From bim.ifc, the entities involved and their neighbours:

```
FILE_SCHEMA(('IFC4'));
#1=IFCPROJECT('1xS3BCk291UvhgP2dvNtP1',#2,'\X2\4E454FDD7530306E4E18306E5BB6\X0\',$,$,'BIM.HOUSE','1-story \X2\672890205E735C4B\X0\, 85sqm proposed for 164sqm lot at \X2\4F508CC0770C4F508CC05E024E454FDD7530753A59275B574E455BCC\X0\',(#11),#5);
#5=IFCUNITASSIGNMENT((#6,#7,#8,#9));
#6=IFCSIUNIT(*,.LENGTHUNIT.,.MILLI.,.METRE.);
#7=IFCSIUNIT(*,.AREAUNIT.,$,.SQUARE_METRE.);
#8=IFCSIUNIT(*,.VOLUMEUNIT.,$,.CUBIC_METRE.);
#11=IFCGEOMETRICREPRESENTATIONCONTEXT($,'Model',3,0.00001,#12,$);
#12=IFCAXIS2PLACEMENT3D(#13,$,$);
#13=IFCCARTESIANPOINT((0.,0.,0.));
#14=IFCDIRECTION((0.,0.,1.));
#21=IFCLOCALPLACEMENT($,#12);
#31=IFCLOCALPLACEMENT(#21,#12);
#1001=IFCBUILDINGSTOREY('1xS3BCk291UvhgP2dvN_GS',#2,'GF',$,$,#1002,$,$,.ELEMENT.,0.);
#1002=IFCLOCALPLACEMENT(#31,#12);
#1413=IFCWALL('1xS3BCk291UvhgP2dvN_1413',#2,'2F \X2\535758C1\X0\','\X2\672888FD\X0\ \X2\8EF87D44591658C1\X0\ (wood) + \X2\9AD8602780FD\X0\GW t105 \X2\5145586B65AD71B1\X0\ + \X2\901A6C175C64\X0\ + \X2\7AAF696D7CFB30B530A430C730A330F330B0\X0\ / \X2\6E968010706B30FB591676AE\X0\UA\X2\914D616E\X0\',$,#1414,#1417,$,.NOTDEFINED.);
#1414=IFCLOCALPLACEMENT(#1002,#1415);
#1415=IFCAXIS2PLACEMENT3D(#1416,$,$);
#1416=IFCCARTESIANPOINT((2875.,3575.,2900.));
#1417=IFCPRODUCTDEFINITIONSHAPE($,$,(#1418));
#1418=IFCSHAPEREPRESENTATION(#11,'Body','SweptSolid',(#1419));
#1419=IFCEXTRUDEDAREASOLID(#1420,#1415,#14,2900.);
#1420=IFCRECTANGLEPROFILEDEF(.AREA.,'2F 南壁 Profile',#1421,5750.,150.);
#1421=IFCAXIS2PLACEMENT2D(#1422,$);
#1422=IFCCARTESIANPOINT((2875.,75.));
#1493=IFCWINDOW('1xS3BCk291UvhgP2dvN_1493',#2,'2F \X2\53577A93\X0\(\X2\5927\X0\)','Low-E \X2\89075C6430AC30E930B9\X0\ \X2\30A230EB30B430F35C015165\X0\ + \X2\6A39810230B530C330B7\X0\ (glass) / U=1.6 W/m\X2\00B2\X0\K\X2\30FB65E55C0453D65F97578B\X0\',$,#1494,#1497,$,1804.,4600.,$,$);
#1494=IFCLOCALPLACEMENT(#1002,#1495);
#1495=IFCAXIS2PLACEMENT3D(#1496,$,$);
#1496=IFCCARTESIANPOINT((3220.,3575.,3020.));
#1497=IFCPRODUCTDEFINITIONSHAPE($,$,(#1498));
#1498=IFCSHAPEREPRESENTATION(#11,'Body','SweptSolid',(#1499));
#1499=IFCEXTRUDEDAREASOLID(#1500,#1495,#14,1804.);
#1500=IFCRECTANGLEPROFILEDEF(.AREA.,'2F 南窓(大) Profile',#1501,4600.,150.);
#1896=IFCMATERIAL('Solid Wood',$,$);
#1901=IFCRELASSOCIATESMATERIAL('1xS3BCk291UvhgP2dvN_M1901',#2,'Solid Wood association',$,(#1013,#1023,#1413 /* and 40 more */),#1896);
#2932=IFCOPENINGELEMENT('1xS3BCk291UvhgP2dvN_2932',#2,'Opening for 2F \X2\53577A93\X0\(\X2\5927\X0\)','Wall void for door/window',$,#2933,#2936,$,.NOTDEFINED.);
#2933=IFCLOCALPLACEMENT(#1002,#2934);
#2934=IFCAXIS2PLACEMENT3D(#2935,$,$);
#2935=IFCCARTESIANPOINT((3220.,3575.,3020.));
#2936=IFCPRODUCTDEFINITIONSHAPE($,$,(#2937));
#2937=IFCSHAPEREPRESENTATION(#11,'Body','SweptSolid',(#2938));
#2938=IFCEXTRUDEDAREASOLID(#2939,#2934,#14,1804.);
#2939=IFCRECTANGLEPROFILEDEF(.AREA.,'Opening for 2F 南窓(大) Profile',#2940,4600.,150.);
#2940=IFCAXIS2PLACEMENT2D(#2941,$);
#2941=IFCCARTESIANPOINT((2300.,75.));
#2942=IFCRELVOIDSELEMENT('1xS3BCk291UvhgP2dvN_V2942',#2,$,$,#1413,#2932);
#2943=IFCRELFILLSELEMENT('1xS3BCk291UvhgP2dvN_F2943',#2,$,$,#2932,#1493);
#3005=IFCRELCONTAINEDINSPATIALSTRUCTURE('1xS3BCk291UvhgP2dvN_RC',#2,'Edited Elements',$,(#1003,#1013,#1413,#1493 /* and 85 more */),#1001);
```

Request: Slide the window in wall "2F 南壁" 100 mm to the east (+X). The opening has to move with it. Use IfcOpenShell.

```python
import ifcopenshell
import ifcopenshell.api.geometry
import ifcopenshell.util.placement

model = ifcopenshell.open("bim.ifc")

window = model.by_guid("1xS3BCk291UvhgP2dvN_1493")
opening = window.FillsVoids[0].RelatingOpeningElement
wall = opening.VoidsElements[0].RelatingBuildingElement

wall_matrix = ifcopenshell.util.placement.get_local_placement(wall.ObjectPlacement)
shift = wall_matrix[:3, 0] * 100.0
before = ifcopenshell.util.placement.get_local_placement(window.ObjectPlacement)[:3, 3].copy()

# The window is not placed relative to its opening, so move both.
for product in (opening, window):
    matrix = ifcopenshell.util.placement.get_local_placement(product.ObjectPlacement)
    matrix[:3, 3] += shift
    ifcopenshell.api.geometry.edit_object_placement(model, product=product, matrix=matrix, is_si=False)

after = ifcopenshell.util.placement.get_local_placement(window.ObjectPlacement)[:3, 3]
print("window moved by", (after - before).round(3) + 0.0)

model.write("bim_edited.ifc")
```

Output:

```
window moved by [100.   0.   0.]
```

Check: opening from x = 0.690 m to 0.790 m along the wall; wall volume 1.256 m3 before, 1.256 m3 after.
